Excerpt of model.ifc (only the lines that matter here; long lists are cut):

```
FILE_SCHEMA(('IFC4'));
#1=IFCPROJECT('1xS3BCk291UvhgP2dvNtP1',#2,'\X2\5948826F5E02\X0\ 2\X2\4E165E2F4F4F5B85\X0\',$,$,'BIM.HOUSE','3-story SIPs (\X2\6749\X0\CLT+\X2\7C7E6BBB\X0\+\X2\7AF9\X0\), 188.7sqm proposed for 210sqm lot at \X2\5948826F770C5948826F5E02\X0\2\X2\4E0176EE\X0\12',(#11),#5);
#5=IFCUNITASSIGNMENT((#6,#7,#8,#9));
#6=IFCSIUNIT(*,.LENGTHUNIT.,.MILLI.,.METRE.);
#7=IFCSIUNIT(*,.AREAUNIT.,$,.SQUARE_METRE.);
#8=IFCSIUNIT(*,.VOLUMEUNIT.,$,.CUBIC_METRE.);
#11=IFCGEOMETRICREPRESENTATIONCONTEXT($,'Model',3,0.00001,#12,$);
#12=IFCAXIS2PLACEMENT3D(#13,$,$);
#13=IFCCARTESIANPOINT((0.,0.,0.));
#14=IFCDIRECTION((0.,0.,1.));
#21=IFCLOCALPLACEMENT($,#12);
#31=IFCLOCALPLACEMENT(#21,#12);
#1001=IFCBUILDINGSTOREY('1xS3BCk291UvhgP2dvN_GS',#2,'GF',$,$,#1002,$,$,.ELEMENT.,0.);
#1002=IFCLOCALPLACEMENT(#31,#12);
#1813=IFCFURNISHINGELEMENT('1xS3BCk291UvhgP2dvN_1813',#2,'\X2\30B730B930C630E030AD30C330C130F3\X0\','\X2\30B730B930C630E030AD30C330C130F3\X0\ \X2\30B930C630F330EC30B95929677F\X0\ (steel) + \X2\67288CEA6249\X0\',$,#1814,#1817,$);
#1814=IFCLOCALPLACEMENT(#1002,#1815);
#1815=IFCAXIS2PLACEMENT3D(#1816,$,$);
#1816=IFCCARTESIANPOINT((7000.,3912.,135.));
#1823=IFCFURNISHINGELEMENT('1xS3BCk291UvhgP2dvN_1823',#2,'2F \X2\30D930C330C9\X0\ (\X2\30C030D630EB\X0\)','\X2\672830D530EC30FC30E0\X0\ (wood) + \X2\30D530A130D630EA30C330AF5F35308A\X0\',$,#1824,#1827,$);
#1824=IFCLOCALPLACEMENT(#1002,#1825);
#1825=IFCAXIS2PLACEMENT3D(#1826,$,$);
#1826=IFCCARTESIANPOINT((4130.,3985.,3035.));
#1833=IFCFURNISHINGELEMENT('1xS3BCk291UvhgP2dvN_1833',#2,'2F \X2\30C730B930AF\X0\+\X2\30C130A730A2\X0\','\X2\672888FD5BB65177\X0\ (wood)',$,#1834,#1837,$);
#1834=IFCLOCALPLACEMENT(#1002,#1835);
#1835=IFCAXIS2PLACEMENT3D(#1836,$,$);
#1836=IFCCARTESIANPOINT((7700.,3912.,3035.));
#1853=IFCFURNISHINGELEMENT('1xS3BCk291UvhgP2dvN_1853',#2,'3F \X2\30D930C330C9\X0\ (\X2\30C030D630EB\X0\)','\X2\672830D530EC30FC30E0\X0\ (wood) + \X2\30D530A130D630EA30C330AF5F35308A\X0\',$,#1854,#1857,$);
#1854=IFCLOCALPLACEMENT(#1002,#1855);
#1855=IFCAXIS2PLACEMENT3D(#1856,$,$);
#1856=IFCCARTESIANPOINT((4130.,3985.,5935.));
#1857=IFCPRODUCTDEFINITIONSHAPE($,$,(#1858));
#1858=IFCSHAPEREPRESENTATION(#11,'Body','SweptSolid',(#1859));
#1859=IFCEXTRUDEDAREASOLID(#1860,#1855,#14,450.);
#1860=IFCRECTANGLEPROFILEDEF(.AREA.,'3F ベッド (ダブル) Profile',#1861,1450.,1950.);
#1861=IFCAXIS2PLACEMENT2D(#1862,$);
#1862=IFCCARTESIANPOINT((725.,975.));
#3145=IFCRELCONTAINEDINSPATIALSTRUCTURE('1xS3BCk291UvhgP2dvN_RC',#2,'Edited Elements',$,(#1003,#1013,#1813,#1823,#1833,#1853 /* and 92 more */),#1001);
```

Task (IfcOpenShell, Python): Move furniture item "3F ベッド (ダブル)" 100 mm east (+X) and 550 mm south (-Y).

```python
import ifcopenshell
import ifcopenshell.api.geometry
import ifcopenshell.util.placement

model = ifcopenshell.open("model.ifc")

item = model.by_guid("1xS3BCk291UvhgP2dvN_1853")
matrix = ifcopenshell.util.placement.get_local_placement(item.ObjectPlacement)
matrix[0, 3] += 100.0
matrix[1, 3] -= 550.0
ifcopenshell.api.geometry.edit_object_placement(model, product=item, matrix=matrix, is_si=False)

print(ifcopenshell.util.placement.get_local_placement(item.ObjectPlacement).round(3) + 0.0)

model.write("model_v2.ifc")
```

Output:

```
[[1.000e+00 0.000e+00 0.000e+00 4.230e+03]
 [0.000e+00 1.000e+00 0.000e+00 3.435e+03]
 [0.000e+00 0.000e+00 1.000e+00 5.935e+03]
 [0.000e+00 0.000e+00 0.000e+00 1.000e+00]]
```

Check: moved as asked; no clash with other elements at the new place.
